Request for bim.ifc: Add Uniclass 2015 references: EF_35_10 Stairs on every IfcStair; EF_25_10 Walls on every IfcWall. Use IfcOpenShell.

First a look at what the model holds.

```python
import ifcopenshell

model = ifcopenshell.open("bim.ifc")
print(model.schema)
print("classifications:", [c.Name for c in model.by_type("IfcClassification")])
for ifc_class in ("IfcDoor", "IfcRoof", "IfcStair", "IfcWall", "IfcWindow"):
    print(ifc_class, len(model.by_type(ifc_class)))
```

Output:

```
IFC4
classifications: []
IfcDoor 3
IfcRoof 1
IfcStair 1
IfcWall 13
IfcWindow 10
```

```python
import ifcopenshell
import ifcopenshell.api.classification

model = ifcopenshell.open("bim.ifc")

system = ifcopenshell.api.classification.add_classification(model, classification="Uniclass 2015")

codes = {
    "IfcStair": ("EF_35_10", "Stairs"),
    "IfcWall": ("EF_25_10", "Walls"),
}
for ifc_class, (code, name) in codes.items():
    products = model.by_type(ifc_class)
    ifcopenshell.api.classification.add_reference(
        model, products=products, classification=system, identification=code, name=name
    )
    print(code, len(products))

model.write("bim_updated.ifc")
```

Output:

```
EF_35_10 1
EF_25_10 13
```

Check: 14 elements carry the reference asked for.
